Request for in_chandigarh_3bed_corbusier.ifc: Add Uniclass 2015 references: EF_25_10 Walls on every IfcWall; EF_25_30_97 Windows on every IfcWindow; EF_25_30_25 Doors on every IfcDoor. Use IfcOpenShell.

First a look at what the model holds.

```python
import ifcopenshell

model = ifcopenshell.open("in_chandigarh_3bed_corbusier.ifc")
print(model.schema)
print("classifications:", [c.Name for c in model.by_type("IfcClassification")])
for ifc_class in ("IfcDoor", "IfcRoof", "IfcStair", "IfcWall", "IfcWindow"):
    print(ifc_class, len(model.by_type(ifc_class)))
```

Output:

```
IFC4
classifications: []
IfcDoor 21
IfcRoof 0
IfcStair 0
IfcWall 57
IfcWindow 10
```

```python
import ifcopenshell
import ifcopenshell.api.classification

model = ifcopenshell.open("in_chandigarh_3bed_corbusier.ifc")

system = ifcopenshell.api.classification.add_classification(model, classification="Uniclass 2015")

codes = {
    "IfcWall": ("EF_25_10", "Walls"),
    "IfcWindow": ("EF_25_30_97", "Windows"),
    "IfcDoor": ("EF_25_30_25", "Doors"),
}
for ifc_class, (code, name) in codes.items():
    products = model.by_type(ifc_class)
    ifcopenshell.api.classification.add_reference(
        model, products=products, classification=system, identification=code, name=name
    )
    print(code, len(products))

model.write("in_chandigarh_3bed_corbusier-out.ifc")
```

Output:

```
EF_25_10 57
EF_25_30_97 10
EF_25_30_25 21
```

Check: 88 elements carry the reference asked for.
